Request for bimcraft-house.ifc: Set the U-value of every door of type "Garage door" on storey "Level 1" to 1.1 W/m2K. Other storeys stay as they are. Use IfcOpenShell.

First a look at what the model holds.

```python
import ifcopenshell
import ifcopenshell.util.element

model = ifcopenshell.open("bimcraft-house.ifc")
print(model.schema)
storey = next(s for s in model.by_type("IfcBuildingStorey") if s.Name == "Level 1")
doors = [e for e in ifcopenshell.util.element.get_decomposition(storey) if e.is_a("IfcDoor")]
seen = {}
for e in doors:
    element_type = ifcopenshell.util.element.get_type(e)
    key = (element_type.Name if element_type != e and element_type else None, ifcopenshell.util.element.get_pset(e, "Pset_DoorCommon", "ThermalTransmittance"))
    seen[key] = seen.get(key, 0) + 1
for (name, value), count in sorted(seen.items(), key=str):
    print(count, "x", name, "|", value)
```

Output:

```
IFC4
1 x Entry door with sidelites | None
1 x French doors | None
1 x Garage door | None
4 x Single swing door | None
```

```python
import ifcopenshell
import ifcopenshell.api.pset
import ifcopenshell.util.element

model = ifcopenshell.open("bimcraft-house.ifc")

storey = next(s for s in model.by_type("IfcBuildingStorey") if s.Name == "Level 1")
doors = [e for e in ifcopenshell.util.element.get_decomposition(storey) if e.is_a("IfcDoor")]

count = 0
for e in doors:
    element_type = ifcopenshell.util.element.get_type(e)
    if element_type in (None, e) or element_type.Name != "Garage door":
        continue
    # add_pset returns the element's existing set when there is one.
    pset = ifcopenshell.api.pset.add_pset(model, product=e, name="Pset_DoorCommon")
    ifcopenshell.api.pset.edit_pset(model, pset=pset, properties={"ThermalTransmittance": 1.1})
    count += 1

print(count, "doors updated")

model.write("bimcraft-house_rev.ifc")
```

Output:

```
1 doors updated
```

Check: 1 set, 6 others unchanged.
